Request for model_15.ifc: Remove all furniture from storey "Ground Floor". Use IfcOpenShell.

First a look at what the model holds.

```python
import ifcopenshell
import ifcopenshell.util.element

model = ifcopenshell.open("model_15.ifc")
print(model.schema)
storey = next(s for s in model.by_type("IfcBuildingStorey") if s.Name == "Ground Floor")
furniture = [e for e in ifcopenshell.util.element.get_decomposition(storey) if e.is_a("IfcFurnishingElement")]
seen = {}
for e in furniture:
    element_type = ifcopenshell.util.element.get_type(e)
    name = element_type.Name if element_type not in (None, e) else None
    seen[name] = seen.get(name, 0) + 1
for name, count in sorted(seen.items(), key=str):
    print(count, "x", name)
```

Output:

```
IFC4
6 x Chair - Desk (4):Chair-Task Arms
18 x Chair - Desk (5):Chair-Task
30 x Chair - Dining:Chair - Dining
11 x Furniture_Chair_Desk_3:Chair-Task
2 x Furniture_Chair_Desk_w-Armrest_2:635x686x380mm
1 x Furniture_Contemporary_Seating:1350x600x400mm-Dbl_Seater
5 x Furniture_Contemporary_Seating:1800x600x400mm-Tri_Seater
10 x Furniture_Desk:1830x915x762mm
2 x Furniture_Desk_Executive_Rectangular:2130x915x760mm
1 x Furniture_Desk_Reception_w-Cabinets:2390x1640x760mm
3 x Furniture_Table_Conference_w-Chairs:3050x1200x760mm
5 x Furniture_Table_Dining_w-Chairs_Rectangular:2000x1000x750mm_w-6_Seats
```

```python
import ifcopenshell
import ifcopenshell.api.root
import ifcopenshell.util.element

model = ifcopenshell.open("model_15.ifc")

storey = next(s for s in model.by_type("IfcBuildingStorey") if s.Name == "Ground Floor")
furniture = [e for e in ifcopenshell.util.element.get_decomposition(storey) if e.is_a("IfcFurnishingElement")]

for e in furniture:
    ifcopenshell.api.root.remove_product(model, product=e)
print(len(furniture), "removed")

model.write("model_15_rev.ifc")
```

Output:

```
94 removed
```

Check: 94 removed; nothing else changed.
